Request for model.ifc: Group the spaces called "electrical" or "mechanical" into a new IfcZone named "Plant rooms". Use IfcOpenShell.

First a look at what the model holds.

```python
import ifcopenshell

model = ifcopenshell.open("model.ifc")
print(model.schema)
seen = {}
for space in model.by_type("IfcSpace"):
    seen[space.LongName] = seen.get(space.LongName, 0) + 1
for name, count in sorted(seen.items(), key=str):
    print(count, "x", name)
print("zones:", [z.Name for z in model.by_type("IfcZone")][:20])
```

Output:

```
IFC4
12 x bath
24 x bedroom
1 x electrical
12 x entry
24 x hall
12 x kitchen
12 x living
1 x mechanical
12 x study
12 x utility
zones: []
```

```python
import ifcopenshell
import ifcopenshell.api.group
import ifcopenshell.api.root

model = ifcopenshell.open("model.ifc")

names = {"electrical", "mechanical"}
spaces = [s for s in model.by_type("IfcSpace") if s.LongName in names]

zone = ifcopenshell.api.root.create_entity(model, ifc_class="IfcZone", name="Plant rooms")
ifcopenshell.api.group.assign_group(model, products=spaces, group=zone)
print(len(spaces), "spaces in", zone.Name)

model.write("model_edited.ifc")
```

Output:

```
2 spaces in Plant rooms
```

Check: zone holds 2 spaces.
